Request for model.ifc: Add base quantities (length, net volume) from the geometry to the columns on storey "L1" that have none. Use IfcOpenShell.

First a look at what the model holds.

```python
import ifcopenshell
import ifcopenshell.util.element
import ifcopenshell.util.unit

model = ifcopenshell.open("model.ifc")
print(model.schema)
for unit_type in ("LENGTHUNIT", "AREAUNIT", "VOLUMEUNIT"):
    print(unit_type, ifcopenshell.util.unit.calculate_unit_scale(model, unit_type))
storey = next(s for s in model.by_type("IfcBuildingStorey") if s.Name == "L1")
columns = [e for e in ifcopenshell.util.element.get_decomposition(storey) if e.is_a("IfcColumn")]
for e in sorted(columns, key=lambda e: e.id()):
    print(e.id(), e.is_a(), e.Name, list(ifcopenshell.util.element.get_psets(e, qtos_only=True)), sep=" | ")
```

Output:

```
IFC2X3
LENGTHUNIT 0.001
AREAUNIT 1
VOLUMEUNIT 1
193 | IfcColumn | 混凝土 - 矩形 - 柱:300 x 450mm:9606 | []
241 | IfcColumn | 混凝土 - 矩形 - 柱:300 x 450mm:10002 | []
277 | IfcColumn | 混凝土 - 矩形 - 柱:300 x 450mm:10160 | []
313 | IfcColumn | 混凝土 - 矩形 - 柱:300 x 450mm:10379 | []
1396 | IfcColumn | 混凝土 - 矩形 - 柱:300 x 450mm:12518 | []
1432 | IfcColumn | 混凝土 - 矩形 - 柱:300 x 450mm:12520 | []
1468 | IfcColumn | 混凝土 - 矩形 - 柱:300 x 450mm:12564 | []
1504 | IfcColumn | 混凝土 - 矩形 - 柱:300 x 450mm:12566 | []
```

```python
import ifcopenshell
import ifcopenshell.api.pset
import ifcopenshell.geom
import ifcopenshell.util.element
import ifcopenshell.util.shape
import ifcopenshell.util.unit

model = ifcopenshell.open("model.ifc")
unit_scale = ifcopenshell.util.unit.calculate_unit_scale(model)
volume_scale = ifcopenshell.util.unit.calculate_unit_scale(model, "VOLUMEUNIT")
settings = ifcopenshell.geom.settings()

storey = next(s for s in model.by_type("IfcBuildingStorey") if s.Name == "L1")
columns = [e for e in ifcopenshell.util.element.get_decomposition(storey) if e.is_a("IfcColumn")]

for e in sorted(columns, key=lambda e: e.id()):
    if ifcopenshell.util.element.get_psets(e, qtos_only=True, should_inherit=False):
        continue
    # Geometry comes back in metres, in the element's own axes.
    shape = ifcopenshell.geom.create_shape(settings, e)
    values = {
        "Length": ifcopenshell.util.shape.get_z(shape.geometry) / unit_scale,
        "NetVolume": ifcopenshell.util.shape.get_volume(shape.geometry) / volume_scale,
    }
    qto = ifcopenshell.api.pset.add_qto(model, product=e, name="BaseQuantities")
    ifcopenshell.api.pset.edit_qto(model, qto=qto, properties=values)
    print(e.id(), {k: round(v, 3) for k, v in values.items()})

model.write("model-out.ifc")
```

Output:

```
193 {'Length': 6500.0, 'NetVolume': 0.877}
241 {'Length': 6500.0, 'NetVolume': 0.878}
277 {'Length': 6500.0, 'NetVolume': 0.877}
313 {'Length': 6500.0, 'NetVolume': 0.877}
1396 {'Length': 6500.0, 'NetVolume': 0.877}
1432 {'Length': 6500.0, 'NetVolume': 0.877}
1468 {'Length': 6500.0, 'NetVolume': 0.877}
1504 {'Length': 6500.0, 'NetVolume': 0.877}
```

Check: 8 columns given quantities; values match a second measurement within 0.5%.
